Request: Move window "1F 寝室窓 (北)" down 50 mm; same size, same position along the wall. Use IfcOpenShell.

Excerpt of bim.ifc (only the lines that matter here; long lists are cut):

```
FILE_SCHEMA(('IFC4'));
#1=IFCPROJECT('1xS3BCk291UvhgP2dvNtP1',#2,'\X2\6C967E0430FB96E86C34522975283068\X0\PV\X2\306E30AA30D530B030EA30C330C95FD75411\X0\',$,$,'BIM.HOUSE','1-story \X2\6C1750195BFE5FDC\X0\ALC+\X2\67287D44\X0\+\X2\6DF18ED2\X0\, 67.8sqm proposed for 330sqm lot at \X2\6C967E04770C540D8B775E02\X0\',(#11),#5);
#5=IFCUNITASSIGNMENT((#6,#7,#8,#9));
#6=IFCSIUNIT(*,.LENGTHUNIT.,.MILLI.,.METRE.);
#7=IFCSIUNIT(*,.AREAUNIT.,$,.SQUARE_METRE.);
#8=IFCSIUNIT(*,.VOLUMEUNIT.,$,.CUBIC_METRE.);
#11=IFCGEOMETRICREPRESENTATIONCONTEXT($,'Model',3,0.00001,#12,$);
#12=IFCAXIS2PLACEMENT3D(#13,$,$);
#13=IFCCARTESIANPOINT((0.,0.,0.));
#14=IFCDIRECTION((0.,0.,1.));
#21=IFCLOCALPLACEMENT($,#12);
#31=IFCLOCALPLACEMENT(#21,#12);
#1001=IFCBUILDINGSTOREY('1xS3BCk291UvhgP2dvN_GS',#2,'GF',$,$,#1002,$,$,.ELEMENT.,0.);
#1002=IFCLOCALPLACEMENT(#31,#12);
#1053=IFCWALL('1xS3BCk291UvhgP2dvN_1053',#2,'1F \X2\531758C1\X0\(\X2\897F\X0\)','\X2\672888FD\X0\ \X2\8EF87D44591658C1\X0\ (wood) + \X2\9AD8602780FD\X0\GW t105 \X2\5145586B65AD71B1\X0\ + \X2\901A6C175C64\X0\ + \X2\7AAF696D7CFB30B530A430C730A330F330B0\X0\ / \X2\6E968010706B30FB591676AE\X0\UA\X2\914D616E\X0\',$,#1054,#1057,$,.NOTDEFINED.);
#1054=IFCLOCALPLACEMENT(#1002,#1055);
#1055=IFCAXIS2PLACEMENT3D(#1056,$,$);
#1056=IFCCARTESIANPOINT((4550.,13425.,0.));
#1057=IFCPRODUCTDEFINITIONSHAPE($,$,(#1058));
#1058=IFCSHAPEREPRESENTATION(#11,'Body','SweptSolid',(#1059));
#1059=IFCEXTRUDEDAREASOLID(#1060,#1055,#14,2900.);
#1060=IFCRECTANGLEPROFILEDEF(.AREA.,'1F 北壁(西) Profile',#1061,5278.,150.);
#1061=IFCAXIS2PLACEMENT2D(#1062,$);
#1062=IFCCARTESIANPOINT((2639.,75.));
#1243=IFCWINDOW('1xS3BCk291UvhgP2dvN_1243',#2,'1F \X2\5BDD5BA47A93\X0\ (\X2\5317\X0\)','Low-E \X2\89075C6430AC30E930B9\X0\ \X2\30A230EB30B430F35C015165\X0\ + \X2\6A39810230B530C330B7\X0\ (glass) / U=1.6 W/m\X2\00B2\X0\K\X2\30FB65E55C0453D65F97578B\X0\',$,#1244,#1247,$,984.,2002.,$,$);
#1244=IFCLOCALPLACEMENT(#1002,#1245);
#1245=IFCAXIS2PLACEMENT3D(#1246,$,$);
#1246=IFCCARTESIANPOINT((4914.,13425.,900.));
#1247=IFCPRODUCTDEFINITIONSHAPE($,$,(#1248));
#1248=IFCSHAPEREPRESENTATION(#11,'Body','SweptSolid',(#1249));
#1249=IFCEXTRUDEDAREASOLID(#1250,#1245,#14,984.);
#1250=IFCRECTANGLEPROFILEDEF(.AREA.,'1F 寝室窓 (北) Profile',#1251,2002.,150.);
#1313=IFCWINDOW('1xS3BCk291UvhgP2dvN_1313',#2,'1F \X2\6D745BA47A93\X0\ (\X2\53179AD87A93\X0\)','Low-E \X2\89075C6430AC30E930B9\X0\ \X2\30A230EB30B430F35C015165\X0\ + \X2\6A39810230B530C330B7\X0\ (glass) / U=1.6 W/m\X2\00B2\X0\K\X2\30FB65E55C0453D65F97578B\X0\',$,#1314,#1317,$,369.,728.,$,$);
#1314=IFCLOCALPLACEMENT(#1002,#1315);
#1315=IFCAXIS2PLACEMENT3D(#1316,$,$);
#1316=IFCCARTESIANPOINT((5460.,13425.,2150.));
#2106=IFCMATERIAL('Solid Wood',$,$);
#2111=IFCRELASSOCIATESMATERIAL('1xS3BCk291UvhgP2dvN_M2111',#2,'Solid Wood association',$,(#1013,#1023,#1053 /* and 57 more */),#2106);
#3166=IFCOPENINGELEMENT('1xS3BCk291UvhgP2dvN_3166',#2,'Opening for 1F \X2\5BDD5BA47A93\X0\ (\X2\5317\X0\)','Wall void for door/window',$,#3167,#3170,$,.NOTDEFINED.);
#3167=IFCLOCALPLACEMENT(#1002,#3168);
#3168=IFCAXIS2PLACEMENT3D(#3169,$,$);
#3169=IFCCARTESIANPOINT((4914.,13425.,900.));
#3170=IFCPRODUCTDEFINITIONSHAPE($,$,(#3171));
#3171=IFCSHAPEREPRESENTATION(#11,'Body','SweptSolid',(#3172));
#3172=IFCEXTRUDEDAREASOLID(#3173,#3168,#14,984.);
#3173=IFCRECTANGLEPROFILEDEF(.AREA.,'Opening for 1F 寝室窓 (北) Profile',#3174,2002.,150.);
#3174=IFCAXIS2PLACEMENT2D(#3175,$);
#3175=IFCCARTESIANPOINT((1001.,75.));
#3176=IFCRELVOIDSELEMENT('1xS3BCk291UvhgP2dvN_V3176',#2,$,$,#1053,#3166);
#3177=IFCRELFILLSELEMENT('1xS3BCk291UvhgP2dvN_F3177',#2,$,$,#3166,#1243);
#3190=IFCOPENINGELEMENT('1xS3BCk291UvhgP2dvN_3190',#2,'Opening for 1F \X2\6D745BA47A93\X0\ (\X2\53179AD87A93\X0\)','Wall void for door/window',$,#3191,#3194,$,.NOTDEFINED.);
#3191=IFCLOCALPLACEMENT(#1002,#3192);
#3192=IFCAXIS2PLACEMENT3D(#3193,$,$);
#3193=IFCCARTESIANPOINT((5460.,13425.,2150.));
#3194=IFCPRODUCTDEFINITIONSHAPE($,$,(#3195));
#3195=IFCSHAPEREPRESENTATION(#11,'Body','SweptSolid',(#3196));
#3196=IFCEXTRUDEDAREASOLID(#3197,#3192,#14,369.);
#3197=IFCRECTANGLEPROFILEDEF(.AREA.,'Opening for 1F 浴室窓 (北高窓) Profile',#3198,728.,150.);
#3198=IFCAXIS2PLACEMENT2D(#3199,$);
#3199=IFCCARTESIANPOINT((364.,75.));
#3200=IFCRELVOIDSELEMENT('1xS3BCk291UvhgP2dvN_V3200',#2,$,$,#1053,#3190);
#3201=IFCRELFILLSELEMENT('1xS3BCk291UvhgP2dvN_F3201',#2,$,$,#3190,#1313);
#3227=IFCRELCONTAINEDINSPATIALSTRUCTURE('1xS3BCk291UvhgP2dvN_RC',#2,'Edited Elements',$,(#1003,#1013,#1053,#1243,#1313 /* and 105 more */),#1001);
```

```python
import numpy as np
import ifcopenshell
import ifcopenshell.api.geometry
import ifcopenshell.util.placement
import ifcopenshell.util.unit

model = ifcopenshell.open("bim.ifc")
unit_scale = ifcopenshell.util.unit.calculate_unit_scale(model)

window = model.by_guid("1xS3BCk291UvhgP2dvN_1243")
opening = window.FillsVoids[0].RelatingOpeningElement
dz = -50.0

shift = np.array([0.0, 0.0, dz])
# The window is not placed relative to its opening, so move both.
for product in (opening, window):
    matrix = ifcopenshell.util.placement.get_local_placement(product.ObjectPlacement)
    matrix[:3, 3] += shift
    ifcopenshell.api.geometry.edit_object_placement(model, product=product, matrix=matrix, is_si=False)

print(f"moved by {dz * unit_scale:+.3f} m")

model.write("bim-out.ifc")
```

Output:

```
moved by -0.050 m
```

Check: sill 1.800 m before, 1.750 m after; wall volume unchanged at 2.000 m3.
